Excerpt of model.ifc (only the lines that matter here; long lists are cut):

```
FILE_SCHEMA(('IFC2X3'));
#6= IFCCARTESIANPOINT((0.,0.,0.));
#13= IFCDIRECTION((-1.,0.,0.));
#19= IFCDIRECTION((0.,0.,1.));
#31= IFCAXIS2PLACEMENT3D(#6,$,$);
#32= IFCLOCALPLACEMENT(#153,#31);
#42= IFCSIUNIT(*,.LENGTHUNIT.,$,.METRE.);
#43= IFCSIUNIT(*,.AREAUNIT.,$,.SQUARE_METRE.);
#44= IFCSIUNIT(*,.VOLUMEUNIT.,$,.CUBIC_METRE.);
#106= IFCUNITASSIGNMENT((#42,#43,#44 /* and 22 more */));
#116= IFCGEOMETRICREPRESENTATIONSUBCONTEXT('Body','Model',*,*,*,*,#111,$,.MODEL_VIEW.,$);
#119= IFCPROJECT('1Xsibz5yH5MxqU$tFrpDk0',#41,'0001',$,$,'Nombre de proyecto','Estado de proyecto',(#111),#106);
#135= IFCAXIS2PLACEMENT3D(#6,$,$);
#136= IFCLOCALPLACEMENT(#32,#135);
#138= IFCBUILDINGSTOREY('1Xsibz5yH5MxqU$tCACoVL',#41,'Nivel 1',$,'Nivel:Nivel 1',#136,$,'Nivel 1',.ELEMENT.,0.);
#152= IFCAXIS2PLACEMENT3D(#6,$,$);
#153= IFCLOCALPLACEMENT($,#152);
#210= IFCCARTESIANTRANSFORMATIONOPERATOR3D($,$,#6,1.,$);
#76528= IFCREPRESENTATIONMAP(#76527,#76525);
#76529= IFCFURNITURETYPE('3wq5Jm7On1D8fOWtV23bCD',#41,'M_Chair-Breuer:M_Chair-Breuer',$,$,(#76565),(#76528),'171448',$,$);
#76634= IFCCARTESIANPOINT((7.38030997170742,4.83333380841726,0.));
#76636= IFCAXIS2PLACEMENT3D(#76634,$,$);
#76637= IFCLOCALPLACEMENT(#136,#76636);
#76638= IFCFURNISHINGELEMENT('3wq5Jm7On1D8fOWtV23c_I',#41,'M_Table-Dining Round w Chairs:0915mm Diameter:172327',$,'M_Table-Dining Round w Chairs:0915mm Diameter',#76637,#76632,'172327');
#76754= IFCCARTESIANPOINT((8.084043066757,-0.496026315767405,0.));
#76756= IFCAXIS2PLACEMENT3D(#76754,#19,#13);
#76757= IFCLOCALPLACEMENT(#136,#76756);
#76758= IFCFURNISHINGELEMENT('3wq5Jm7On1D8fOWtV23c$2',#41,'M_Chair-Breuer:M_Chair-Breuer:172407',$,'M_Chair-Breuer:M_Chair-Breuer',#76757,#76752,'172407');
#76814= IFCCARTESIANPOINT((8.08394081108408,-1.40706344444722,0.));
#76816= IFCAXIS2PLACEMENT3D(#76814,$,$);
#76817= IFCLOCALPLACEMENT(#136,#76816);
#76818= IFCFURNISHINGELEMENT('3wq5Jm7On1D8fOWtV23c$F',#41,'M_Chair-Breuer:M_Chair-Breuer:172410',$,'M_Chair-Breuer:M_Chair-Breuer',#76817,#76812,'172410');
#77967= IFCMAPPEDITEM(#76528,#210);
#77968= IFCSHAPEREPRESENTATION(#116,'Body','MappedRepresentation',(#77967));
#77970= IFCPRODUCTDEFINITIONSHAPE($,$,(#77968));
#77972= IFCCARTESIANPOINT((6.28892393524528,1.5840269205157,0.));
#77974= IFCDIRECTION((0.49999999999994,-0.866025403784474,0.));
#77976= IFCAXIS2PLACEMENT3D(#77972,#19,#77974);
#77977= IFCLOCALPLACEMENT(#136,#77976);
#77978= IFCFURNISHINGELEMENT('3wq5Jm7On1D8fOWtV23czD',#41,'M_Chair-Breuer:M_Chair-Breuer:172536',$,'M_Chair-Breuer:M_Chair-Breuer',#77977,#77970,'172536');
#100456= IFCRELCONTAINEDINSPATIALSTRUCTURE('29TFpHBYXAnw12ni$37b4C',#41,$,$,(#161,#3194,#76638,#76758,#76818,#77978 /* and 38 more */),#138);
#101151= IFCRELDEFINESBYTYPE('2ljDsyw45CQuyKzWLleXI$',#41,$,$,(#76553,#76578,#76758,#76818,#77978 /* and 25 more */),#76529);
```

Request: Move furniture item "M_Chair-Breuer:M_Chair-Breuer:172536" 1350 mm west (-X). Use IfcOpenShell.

```python
import ifcopenshell
import ifcopenshell.api.geometry
import ifcopenshell.util.placement
import ifcopenshell.util.unit

model = ifcopenshell.open("model.ifc")
unit_scale = ifcopenshell.util.unit.calculate_unit_scale(model)

item = model.by_id(77978)
matrix = ifcopenshell.util.placement.get_local_placement(item.ObjectPlacement)
matrix[0, 3] -= 1.35 / unit_scale
ifcopenshell.api.geometry.edit_object_placement(model, product=item, matrix=matrix, is_si=False)

print(ifcopenshell.util.placement.get_local_placement(item.ObjectPlacement).round(3) + 0.0)

model.write("model_updated.ifc")
```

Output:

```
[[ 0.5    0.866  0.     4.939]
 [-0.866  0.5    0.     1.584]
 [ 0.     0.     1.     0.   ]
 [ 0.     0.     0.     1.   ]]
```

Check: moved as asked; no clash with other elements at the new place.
